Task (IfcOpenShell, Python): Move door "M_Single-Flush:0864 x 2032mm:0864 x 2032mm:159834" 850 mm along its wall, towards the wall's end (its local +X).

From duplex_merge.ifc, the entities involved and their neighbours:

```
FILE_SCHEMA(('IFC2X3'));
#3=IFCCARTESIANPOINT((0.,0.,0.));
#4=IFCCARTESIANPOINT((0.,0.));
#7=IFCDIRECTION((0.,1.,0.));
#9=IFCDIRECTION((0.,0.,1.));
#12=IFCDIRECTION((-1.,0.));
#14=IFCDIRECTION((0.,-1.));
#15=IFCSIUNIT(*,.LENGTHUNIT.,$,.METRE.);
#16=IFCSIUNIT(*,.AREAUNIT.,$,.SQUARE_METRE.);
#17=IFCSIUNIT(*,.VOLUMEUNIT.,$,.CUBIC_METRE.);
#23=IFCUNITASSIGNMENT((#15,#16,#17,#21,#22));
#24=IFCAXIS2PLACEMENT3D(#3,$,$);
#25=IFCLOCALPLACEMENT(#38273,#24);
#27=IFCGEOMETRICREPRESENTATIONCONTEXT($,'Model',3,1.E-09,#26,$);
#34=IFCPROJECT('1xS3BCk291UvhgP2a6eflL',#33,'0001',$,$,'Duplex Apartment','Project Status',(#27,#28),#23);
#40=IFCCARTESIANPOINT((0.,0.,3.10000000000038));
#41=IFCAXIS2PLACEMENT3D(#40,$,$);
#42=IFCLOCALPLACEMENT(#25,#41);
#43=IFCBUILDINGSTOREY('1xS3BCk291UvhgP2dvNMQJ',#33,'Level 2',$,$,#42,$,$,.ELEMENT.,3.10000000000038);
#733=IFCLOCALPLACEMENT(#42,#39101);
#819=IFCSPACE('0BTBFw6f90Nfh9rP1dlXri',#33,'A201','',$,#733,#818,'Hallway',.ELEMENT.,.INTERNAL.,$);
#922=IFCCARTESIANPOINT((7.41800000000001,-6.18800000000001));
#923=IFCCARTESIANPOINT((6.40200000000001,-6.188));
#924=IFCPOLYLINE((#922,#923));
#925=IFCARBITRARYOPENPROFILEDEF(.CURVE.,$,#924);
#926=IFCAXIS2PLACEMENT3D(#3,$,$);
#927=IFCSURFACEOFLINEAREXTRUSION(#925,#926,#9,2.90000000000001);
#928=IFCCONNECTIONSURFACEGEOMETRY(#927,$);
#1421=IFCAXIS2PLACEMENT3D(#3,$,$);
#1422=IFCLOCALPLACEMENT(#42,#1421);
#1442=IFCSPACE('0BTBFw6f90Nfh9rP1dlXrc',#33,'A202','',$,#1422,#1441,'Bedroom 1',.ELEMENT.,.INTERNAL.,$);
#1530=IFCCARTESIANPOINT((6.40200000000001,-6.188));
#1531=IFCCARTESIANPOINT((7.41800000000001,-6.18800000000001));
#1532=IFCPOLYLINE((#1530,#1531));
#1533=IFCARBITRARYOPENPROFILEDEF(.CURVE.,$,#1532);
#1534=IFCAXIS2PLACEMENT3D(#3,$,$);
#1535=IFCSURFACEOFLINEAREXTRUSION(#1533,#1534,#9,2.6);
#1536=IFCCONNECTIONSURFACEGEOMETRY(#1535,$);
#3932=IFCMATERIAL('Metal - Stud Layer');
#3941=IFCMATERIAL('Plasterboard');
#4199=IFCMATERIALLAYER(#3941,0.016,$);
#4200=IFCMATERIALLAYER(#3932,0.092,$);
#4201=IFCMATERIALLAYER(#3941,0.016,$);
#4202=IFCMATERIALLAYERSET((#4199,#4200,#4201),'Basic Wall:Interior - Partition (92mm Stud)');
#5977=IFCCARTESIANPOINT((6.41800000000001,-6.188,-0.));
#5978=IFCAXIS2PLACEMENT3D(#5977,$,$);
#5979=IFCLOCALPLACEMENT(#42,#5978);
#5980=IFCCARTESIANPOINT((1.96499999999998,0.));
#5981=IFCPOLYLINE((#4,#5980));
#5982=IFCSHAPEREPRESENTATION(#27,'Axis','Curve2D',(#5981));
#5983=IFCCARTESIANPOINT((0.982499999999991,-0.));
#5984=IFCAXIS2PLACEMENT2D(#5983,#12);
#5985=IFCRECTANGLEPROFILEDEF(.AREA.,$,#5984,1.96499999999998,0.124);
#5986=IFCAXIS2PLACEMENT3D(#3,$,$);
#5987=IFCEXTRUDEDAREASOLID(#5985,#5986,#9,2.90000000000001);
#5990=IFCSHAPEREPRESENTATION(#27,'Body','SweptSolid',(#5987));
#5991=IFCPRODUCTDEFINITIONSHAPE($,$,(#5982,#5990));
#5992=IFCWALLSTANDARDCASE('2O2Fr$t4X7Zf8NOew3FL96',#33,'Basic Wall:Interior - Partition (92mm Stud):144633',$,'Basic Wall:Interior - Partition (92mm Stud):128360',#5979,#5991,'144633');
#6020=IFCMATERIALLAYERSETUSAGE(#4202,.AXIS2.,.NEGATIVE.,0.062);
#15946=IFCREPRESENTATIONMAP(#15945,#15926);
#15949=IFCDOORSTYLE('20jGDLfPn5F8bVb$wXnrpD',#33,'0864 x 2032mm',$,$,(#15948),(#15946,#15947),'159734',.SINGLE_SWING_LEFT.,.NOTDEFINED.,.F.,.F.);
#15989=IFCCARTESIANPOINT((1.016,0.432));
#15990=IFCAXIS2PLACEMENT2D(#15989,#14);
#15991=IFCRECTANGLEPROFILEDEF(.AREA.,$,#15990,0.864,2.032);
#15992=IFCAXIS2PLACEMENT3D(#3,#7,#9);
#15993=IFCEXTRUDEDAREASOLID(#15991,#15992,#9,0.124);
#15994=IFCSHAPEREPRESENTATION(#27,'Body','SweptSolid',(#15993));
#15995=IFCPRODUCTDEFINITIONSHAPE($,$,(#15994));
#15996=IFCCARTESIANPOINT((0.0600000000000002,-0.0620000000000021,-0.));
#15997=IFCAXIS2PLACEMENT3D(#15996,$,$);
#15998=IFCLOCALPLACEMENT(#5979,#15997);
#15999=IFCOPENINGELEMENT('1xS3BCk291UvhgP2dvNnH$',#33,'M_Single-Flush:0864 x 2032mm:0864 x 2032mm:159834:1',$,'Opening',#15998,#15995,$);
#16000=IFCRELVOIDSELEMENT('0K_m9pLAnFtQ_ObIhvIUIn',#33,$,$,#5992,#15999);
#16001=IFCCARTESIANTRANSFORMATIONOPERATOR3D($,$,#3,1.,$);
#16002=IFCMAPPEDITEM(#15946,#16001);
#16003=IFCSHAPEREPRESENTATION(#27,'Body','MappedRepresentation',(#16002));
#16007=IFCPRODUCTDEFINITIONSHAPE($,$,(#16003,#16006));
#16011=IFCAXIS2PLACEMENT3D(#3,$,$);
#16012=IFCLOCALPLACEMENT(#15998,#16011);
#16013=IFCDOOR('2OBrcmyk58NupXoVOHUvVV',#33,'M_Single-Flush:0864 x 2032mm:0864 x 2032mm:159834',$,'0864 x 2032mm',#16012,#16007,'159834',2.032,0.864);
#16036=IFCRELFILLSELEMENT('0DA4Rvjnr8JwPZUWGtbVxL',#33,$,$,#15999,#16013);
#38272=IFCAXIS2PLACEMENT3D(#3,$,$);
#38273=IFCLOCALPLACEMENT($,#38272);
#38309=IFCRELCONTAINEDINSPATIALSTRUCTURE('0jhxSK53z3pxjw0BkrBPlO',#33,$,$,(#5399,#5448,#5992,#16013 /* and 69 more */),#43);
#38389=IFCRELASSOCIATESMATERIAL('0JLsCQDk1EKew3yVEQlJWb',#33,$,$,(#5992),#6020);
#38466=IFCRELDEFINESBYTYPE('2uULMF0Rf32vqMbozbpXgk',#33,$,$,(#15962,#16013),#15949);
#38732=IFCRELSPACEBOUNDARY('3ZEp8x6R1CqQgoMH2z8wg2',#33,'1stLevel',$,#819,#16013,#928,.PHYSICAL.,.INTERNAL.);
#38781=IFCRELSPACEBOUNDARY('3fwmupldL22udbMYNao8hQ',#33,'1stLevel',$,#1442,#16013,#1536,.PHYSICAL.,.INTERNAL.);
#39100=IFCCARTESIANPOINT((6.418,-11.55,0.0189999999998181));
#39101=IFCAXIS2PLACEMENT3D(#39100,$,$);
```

```python
import numpy as np
import ifcopenshell
import ifcopenshell.api.geometry
import ifcopenshell.util.placement
import ifcopenshell.util.unit

model = ifcopenshell.open("duplex_merge.ifc")
unit_scale = ifcopenshell.util.unit.calculate_unit_scale(model)

door = model.by_guid("2OBrcmyk58NupXoVOHUvVV")
opening = door.FillsVoids[0].RelatingOpeningElement
wall = opening.VoidsElements[0].RelatingBuildingElement

wall_matrix = ifcopenshell.util.placement.get_local_placement(wall.ObjectPlacement)
shift = wall_matrix[:3, 0] * 0.85 / unit_scale
before = ifcopenshell.util.placement.get_local_placement(door.ObjectPlacement)[:3, 3].copy()

# The door is placed relative to its opening, so it follows when the opening moves.
matrix = ifcopenshell.util.placement.get_local_placement(opening.ObjectPlacement)
matrix[:3, 3] += shift
ifcopenshell.api.geometry.edit_object_placement(
    model, product=opening, matrix=matrix, is_si=False, should_transform_children=True
)

# Space boundary surfaces are stored in each space's coordinates; move them too.
for rel in door.ProvidesBoundaries:
    if not rel.ConnectionGeometry:
        continue
    surface = rel.ConnectionGeometry.SurfaceOnRelatingElement
    space_matrix = ifcopenshell.util.placement.get_local_placement(rel.RelatingSpace.ObjectPlacement)
    point = np.array(surface.Position.Location.Coordinates) + space_matrix[:3, :3].T @ shift
    surface.Position = model.createIfcAxis2Placement3D(
        model.createIfcCartesianPoint(point.tolist()), surface.Position.Axis, surface.Position.RefDirection
    )

after = ifcopenshell.util.placement.get_local_placement(door.ObjectPlacement)[:3, 3]
print("door moved by", (after - before).round(3) + 0.0)

model.write("duplex_merge_rev.ifc")
```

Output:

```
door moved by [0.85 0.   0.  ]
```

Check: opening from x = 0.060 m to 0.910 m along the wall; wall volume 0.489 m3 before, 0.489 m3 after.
